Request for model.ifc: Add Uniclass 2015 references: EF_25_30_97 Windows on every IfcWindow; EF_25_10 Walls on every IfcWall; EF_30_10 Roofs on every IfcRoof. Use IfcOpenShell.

First a look at what the model holds.

```python
import ifcopenshell

model = ifcopenshell.open("model.ifc")
print(model.schema)
print("classifications:", [c.Name for c in model.by_type("IfcClassification")])
for ifc_class in ("IfcDoor", "IfcRoof", "IfcStair", "IfcWall", "IfcWindow"):
    print(ifc_class, len(model.by_type(ifc_class)))
```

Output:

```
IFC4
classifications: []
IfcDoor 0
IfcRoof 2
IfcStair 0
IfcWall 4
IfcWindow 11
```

```python
import ifcopenshell
import ifcopenshell.api.classification

model = ifcopenshell.open("model.ifc")

system = ifcopenshell.api.classification.add_classification(model, classification="Uniclass 2015")

codes = {
    "IfcWindow": ("EF_25_30_97", "Windows"),
    "IfcWall": ("EF_25_10", "Walls"),
    "IfcRoof": ("EF_30_10", "Roofs"),
}
for ifc_class, (code, name) in codes.items():
    products = model.by_type(ifc_class)
    ifcopenshell.api.classification.add_reference(
        model, products=products, classification=system, identification=code, name=name
    )
    print(code, len(products))

model.write("model_v2.ifc")
```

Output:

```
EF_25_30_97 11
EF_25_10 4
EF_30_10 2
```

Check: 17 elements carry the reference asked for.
